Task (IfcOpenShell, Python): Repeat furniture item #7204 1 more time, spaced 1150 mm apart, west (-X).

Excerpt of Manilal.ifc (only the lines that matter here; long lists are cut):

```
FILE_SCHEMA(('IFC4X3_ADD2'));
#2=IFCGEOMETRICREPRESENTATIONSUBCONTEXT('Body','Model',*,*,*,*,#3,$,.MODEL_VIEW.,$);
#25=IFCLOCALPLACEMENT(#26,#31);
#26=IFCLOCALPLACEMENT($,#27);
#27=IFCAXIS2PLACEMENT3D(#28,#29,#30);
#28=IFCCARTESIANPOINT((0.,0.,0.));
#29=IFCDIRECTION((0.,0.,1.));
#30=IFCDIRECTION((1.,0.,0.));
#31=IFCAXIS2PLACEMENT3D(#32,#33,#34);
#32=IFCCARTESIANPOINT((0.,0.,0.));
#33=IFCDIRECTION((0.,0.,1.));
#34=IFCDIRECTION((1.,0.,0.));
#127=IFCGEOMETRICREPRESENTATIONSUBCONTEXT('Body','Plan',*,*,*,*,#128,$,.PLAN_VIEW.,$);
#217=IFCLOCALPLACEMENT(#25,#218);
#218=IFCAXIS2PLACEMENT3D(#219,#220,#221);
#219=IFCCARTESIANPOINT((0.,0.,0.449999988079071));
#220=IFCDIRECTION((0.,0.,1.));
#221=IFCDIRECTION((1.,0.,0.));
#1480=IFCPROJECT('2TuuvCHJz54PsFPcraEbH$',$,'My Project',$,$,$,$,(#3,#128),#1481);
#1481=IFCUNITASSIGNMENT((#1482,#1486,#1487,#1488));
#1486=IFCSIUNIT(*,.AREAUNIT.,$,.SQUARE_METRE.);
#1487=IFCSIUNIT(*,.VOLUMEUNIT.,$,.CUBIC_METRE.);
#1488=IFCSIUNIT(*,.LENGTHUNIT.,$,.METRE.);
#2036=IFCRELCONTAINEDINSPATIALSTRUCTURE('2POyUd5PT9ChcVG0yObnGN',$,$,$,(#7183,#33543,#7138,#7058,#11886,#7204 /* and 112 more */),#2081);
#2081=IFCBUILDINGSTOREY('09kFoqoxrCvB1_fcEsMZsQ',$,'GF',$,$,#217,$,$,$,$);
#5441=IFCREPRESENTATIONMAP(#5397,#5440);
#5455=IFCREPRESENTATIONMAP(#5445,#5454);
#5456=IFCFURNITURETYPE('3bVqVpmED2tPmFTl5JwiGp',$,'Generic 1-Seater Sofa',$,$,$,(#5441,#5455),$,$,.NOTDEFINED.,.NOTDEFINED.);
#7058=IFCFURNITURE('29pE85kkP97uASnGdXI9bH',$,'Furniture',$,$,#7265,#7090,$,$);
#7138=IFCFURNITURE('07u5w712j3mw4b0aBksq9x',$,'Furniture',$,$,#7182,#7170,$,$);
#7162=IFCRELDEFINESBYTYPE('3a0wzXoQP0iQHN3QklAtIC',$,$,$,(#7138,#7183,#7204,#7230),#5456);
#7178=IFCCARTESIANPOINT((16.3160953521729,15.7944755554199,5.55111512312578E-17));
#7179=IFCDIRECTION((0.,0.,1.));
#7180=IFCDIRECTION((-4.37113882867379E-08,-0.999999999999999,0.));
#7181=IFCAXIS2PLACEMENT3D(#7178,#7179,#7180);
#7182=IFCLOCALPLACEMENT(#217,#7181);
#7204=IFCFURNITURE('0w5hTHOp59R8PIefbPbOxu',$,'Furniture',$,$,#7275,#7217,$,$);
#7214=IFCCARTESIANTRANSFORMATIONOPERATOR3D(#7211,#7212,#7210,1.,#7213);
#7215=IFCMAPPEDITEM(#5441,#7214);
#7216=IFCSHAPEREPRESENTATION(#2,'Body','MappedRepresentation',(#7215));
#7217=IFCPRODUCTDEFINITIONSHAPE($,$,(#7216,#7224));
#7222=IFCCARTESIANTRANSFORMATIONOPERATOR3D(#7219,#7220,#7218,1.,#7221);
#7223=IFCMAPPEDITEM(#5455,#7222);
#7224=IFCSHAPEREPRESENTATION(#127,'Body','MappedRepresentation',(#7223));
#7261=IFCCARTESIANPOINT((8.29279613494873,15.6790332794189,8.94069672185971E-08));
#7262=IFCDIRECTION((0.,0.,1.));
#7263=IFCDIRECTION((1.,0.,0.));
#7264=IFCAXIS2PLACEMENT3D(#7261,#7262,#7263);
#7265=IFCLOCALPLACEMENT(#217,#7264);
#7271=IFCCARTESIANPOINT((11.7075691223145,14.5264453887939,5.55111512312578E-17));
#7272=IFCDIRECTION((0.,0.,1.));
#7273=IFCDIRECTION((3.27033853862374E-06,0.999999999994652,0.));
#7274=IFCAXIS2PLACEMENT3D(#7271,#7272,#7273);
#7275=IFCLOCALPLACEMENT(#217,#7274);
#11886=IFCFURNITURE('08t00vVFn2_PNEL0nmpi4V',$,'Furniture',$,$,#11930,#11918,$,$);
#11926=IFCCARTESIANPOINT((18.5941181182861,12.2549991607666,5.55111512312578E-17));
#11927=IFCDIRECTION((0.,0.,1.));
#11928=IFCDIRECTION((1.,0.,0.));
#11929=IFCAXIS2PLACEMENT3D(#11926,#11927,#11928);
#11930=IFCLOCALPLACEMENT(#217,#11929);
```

```python
import numpy as np
import ifcopenshell
import ifcopenshell.api.geometry
import ifcopenshell.api.root
import ifcopenshell.util.element
import ifcopenshell.util.placement
import ifcopenshell.util.unit

model = ifcopenshell.open("Manilal.ifc")
unit_scale = ifcopenshell.util.unit.calculate_unit_scale(model)

source = model.by_id(7204)
base = ifcopenshell.util.placement.get_local_placement(source.ObjectPlacement)
step = np.array([-1.0, 0.0, 0.0]) * 1.15 / unit_scale

for i in range(1, 2):
    copy = ifcopenshell.api.root.copy_class(model, product=source)
    copy.Representation = ifcopenshell.util.element.copy_deep(
        model, source.Representation, exclude=["IfcGeometricRepresentationContext", "IfcRepresentationMap"]
    )
    matrix = base.copy()
    matrix[:3, 3] += i * step
    print("added at", matrix[:3, 3].round(3) + 0.0)
    ifcopenshell.api.geometry.edit_object_placement(model, product=copy, matrix=matrix, is_si=False)

model.write("Manilal-out.ifc")
```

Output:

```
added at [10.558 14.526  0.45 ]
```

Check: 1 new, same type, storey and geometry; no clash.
